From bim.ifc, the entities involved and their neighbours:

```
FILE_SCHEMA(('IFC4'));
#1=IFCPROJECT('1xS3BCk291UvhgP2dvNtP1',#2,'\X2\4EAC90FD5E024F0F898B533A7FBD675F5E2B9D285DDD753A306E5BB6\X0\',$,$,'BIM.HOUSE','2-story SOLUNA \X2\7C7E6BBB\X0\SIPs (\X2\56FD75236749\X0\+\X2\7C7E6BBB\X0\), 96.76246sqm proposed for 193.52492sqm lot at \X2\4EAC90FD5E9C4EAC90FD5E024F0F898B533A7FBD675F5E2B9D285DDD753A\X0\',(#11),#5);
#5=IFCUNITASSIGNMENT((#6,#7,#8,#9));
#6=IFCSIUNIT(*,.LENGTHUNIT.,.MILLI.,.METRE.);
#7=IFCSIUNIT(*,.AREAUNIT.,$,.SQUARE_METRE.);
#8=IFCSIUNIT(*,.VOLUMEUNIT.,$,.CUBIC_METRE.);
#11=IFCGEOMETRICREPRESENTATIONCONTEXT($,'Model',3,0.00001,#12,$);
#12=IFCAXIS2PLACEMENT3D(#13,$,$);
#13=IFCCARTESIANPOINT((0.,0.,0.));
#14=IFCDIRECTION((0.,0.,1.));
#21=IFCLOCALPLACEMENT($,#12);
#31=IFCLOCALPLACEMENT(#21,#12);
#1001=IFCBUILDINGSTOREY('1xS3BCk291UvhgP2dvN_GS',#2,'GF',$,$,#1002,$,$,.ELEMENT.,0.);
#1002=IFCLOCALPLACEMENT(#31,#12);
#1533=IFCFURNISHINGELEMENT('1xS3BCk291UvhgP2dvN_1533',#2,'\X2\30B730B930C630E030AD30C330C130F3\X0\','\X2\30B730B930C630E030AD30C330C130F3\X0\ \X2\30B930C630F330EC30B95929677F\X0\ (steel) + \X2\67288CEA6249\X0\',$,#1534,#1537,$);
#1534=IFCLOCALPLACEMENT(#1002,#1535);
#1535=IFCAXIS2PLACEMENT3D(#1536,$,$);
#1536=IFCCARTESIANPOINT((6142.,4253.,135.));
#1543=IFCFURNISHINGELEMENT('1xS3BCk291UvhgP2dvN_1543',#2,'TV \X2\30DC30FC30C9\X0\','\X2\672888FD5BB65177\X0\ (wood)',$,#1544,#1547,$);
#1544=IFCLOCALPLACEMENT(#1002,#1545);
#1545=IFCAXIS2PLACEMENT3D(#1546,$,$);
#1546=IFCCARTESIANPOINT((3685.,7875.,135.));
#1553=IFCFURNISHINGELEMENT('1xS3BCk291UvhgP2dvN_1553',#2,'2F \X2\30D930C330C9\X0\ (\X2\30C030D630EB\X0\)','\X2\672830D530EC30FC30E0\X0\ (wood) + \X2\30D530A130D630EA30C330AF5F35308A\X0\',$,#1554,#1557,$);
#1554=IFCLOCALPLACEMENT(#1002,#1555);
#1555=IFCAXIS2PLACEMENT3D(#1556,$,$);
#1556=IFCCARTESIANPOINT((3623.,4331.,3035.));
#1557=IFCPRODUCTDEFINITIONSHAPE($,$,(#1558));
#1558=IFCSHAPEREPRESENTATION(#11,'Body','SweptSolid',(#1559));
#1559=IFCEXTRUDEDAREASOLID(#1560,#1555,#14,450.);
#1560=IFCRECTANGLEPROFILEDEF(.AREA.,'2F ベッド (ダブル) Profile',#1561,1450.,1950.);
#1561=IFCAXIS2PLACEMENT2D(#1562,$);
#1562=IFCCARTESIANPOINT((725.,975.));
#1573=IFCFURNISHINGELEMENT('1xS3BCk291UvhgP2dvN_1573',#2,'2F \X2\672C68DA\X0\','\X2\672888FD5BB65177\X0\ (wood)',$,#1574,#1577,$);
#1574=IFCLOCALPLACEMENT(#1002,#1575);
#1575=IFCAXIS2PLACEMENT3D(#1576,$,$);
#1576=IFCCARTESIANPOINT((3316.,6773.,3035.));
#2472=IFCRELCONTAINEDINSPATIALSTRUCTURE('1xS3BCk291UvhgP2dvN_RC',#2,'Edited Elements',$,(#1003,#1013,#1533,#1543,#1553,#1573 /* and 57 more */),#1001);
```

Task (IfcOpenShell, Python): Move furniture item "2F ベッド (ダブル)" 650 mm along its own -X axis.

```python
import ifcopenshell
import ifcopenshell.api.geometry
import ifcopenshell.util.placement
import ifcopenshell.util.unit

model = ifcopenshell.open("bim.ifc")
unit_scale = ifcopenshell.util.unit.calculate_unit_scale(model)

item = model.by_guid("1xS3BCk291UvhgP2dvN_1553")
matrix = ifcopenshell.util.placement.get_local_placement(item.ObjectPlacement)
matrix[:3, 3] -= matrix[:3, 0] * 0.65 / unit_scale
ifcopenshell.api.geometry.edit_object_placement(model, product=item, matrix=matrix, is_si=False)

print(ifcopenshell.util.placement.get_local_placement(item.ObjectPlacement).round(3) + 0.0)

model.write("bim-out.ifc")
```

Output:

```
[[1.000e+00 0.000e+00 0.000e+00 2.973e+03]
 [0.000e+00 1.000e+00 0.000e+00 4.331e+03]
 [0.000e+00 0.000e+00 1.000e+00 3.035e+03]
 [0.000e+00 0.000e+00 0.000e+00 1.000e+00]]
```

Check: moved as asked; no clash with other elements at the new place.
